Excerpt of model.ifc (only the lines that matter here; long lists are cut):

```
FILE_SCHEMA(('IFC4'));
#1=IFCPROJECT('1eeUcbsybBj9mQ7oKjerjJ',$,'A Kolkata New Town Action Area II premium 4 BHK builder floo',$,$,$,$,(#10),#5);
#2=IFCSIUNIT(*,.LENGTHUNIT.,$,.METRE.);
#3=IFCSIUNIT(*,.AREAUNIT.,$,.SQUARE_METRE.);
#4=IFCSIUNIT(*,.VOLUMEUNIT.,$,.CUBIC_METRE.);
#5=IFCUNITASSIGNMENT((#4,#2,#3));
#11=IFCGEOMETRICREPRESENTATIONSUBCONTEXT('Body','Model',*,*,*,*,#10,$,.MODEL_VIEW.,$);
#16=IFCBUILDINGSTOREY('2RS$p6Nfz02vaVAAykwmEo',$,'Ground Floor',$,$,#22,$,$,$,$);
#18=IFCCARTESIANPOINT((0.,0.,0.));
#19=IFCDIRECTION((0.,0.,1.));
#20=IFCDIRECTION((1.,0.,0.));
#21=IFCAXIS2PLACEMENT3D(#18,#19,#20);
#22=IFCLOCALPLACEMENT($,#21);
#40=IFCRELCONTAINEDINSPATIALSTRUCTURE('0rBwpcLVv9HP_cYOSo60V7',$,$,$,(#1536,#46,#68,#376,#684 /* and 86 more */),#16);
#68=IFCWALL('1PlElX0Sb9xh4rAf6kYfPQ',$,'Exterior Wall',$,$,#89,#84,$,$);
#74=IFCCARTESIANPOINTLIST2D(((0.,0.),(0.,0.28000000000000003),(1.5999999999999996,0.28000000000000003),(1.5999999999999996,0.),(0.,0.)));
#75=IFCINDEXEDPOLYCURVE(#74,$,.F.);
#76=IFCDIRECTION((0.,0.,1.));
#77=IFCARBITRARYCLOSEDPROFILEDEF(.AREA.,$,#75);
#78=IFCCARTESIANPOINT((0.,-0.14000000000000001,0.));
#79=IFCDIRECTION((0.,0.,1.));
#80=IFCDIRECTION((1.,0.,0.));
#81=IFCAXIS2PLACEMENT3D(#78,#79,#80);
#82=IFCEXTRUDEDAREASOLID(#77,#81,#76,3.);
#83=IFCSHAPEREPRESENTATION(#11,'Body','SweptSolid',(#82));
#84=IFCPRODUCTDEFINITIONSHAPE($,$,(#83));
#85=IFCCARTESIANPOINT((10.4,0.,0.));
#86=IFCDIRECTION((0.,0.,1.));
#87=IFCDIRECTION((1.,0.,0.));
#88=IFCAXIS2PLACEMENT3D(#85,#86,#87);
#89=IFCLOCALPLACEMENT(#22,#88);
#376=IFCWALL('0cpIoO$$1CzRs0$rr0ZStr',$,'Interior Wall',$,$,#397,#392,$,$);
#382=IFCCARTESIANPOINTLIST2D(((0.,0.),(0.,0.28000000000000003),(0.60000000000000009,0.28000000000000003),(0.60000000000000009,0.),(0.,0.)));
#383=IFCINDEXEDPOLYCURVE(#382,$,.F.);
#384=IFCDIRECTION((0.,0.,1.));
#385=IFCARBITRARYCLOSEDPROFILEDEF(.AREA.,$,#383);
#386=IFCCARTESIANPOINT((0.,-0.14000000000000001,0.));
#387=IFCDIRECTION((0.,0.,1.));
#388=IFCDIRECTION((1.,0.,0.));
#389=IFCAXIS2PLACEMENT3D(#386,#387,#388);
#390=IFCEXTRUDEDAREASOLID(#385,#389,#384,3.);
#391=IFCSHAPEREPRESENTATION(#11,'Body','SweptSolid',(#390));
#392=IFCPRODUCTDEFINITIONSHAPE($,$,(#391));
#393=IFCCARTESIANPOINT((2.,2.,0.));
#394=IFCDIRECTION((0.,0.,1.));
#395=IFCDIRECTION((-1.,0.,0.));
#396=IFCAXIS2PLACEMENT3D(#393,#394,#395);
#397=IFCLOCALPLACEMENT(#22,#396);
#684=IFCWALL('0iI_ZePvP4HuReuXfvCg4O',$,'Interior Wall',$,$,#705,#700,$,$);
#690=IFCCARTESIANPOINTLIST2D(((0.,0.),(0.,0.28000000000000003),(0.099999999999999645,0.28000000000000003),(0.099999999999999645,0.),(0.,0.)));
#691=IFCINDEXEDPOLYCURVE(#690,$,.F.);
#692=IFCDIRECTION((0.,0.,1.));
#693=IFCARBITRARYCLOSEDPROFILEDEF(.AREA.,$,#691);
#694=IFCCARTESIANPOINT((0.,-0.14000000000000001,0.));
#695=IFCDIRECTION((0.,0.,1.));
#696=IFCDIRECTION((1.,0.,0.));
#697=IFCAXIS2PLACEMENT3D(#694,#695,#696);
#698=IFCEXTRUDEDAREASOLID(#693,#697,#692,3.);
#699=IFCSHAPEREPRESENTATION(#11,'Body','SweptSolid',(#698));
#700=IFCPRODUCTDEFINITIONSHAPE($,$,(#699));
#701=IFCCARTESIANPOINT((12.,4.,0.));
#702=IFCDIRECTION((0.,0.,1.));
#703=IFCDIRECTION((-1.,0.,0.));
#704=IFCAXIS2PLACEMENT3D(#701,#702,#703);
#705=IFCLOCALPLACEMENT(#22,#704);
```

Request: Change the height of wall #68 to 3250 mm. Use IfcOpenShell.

```python
import ifcopenshell
import ifcopenshell.geom
import ifcopenshell.util.representation
import ifcopenshell.util.shape

model = ifcopenshell.open("model.ifc")
settings = ifcopenshell.geom.settings()


def volume(element):
    """Net volume in cubic metres, openings subtracted."""
    shape = ifcopenshell.geom.create_shape(settings, element)
    return ifcopenshell.util.shape.get_volume(shape.geometry)


wall = model.by_guid("1PlElX0Sb9xh4rAf6kYfPQ")
before = volume(wall)

body = ifcopenshell.util.representation.get_representation(wall, "Model", "Body")
solid = body.Items[0]
old_height = solid.Depth
solid.Depth = 3.25
after = volume(wall)

print(f"height {old_height:g} -> {solid.Depth:g}, volume {before:.3f} -> {after:.3f} m3")

model.write("model-out.ifc")
```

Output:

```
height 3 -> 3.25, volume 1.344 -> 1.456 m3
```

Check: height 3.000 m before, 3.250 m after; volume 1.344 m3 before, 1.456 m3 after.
